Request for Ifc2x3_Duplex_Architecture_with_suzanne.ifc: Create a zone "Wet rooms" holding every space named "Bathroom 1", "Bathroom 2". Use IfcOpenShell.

First a look at what the model holds.

```python
import ifcopenshell

model = ifcopenshell.open("Ifc2x3_Duplex_Architecture_with_suzanne.ifc")
print(model.schema)
seen = {}
for space in model.by_type("IfcSpace"):
    seen[space.LongName] = seen.get(space.LongName, 0) + 1
for name, count in sorted(seen.items(), key=str):
    print(count, "x", name)
print("zones:", [z.Name for z in model.by_type("IfcZone")][:20])
```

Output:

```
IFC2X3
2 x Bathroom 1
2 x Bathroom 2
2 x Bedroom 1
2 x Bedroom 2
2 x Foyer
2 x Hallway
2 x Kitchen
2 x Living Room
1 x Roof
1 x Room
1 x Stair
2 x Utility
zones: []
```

```python
import ifcopenshell
import ifcopenshell.api.group
import ifcopenshell.api.root

model = ifcopenshell.open("Ifc2x3_Duplex_Architecture_with_suzanne.ifc")

names = {"Bathroom 1", "Bathroom 2"}
spaces = [s for s in model.by_type("IfcSpace") if s.LongName in names]

zone = ifcopenshell.api.root.create_entity(model, ifc_class="IfcZone", name="Wet rooms")
ifcopenshell.api.group.assign_group(model, products=spaces, group=zone)
print(len(spaces), "spaces in", zone.Name)

model.write("Ifc2x3_Duplex_Architecture_with_suzanne-out.ifc")
```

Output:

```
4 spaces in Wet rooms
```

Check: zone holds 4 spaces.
